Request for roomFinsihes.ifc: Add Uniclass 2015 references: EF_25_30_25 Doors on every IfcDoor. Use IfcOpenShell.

First a look at what the model holds.

```python
import ifcopenshell

model = ifcopenshell.open("roomFinsihes.ifc")
print(model.schema)
print("classifications:", [c.Name for c in model.by_type("IfcClassification")])
for ifc_class in ("IfcDoor", "IfcRoof", "IfcStair", "IfcWall", "IfcWindow"):
    print(ifc_class, len(model.by_type(ifc_class)))
```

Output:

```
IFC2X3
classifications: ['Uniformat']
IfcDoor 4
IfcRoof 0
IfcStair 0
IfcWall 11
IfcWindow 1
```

```python
import ifcopenshell
import ifcopenshell.api.classification

model = ifcopenshell.open("roomFinsihes.ifc")

# IFC2X3 requires Source and Edition and has no link from the project to the system.
system = model.create_entity("IfcClassification", Source="NBS", Edition="2015", Name="Uniclass 2015")

codes = {
    "IfcDoor": ("EF_25_30_25", "Doors"),
}
for ifc_class, (code, name) in codes.items():
    products = model.by_type(ifc_class)
    ifcopenshell.api.classification.add_reference(
        model, products=products, classification=system, identification=code, name=name
    )
    print(code, len(products))

model.write("roomFinsihes_updated.ifc")
```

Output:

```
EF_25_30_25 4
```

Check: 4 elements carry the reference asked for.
